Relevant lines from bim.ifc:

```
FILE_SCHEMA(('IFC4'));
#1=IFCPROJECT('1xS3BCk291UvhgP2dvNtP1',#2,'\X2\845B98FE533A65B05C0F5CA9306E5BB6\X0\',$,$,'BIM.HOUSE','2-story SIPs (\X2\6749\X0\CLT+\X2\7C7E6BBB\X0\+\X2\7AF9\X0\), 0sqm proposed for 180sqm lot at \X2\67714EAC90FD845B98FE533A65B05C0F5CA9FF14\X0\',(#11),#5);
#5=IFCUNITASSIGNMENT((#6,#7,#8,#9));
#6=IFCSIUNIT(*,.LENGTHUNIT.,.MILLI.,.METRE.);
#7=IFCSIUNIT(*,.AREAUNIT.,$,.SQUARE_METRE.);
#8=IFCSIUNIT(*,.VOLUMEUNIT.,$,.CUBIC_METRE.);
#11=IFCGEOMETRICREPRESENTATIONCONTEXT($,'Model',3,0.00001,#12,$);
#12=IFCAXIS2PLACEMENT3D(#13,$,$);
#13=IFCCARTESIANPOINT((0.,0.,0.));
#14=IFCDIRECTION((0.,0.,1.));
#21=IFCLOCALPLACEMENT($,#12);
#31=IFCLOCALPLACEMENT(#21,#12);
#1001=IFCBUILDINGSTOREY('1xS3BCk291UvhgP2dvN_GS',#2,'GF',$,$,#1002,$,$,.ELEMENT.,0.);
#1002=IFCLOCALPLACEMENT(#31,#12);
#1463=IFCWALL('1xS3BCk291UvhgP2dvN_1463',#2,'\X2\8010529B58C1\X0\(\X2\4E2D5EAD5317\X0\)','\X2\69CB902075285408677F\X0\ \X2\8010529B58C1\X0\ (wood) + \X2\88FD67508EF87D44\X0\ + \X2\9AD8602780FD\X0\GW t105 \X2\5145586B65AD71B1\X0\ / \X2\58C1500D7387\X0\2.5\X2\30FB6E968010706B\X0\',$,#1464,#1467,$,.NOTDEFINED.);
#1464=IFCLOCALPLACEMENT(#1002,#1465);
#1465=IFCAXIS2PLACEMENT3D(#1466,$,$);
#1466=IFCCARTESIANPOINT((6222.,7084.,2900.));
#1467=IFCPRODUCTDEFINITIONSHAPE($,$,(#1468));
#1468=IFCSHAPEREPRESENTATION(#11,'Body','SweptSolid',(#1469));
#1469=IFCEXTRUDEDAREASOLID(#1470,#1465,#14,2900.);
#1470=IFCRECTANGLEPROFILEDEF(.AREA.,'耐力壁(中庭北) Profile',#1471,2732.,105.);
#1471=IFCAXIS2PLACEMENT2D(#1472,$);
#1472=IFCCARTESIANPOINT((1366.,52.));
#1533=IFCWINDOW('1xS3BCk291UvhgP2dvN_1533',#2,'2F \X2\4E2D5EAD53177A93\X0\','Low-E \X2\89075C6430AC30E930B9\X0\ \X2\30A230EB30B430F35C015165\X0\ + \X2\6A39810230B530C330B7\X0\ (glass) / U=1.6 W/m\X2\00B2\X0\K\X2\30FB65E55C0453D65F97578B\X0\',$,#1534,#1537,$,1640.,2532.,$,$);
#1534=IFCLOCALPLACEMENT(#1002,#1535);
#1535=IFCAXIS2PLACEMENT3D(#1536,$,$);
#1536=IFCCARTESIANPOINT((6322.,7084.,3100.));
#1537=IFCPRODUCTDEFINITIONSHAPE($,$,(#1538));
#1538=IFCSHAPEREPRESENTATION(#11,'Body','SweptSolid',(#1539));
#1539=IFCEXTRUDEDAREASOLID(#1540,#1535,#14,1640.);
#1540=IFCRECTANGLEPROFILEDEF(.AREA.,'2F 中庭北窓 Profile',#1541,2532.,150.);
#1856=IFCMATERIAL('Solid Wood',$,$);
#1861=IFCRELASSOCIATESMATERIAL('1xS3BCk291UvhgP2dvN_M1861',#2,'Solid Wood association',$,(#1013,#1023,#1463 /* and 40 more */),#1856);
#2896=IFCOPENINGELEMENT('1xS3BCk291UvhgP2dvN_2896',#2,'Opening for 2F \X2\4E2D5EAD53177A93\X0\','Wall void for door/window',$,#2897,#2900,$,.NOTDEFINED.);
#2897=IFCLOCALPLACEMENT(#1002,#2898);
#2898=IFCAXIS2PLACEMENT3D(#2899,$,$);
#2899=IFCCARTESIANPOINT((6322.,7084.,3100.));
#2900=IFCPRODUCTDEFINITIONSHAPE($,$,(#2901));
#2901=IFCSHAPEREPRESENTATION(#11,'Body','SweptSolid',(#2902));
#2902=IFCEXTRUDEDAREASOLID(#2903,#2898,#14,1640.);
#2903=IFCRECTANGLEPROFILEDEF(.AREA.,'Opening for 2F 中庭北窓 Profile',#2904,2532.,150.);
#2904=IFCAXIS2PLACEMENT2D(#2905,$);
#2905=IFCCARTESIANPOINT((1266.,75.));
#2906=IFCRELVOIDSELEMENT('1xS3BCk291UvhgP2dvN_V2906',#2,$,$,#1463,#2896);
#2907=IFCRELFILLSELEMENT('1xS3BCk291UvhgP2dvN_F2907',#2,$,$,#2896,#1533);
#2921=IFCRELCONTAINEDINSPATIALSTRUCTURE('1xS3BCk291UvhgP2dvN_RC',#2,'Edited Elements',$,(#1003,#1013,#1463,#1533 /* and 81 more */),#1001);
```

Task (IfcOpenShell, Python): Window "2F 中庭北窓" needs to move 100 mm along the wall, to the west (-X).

```python
import ifcopenshell
import ifcopenshell.api.geometry
import ifcopenshell.util.placement

model = ifcopenshell.open("bim.ifc")

window = model.by_id(1533)
opening = window.FillsVoids[0].RelatingOpeningElement
wall = opening.VoidsElements[0].RelatingBuildingElement

wall_matrix = ifcopenshell.util.placement.get_local_placement(wall.ObjectPlacement)
shift = wall_matrix[:3, 0] * -100.0
before = ifcopenshell.util.placement.get_local_placement(window.ObjectPlacement)[:3, 3].copy()

# The window is not placed relative to its opening, so move both.
for product in (opening, window):
    matrix = ifcopenshell.util.placement.get_local_placement(product.ObjectPlacement)
    matrix[:3, 3] += shift
    ifcopenshell.api.geometry.edit_object_placement(model, product=product, matrix=matrix, is_si=False)

after = ifcopenshell.util.placement.get_local_placement(window.ObjectPlacement)[:3, 3]
print("window moved by", (after - before).round(3) + 0.0)

model.write("bim-out.ifc")
```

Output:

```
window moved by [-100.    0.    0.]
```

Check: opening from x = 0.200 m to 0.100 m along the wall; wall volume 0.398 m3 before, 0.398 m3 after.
